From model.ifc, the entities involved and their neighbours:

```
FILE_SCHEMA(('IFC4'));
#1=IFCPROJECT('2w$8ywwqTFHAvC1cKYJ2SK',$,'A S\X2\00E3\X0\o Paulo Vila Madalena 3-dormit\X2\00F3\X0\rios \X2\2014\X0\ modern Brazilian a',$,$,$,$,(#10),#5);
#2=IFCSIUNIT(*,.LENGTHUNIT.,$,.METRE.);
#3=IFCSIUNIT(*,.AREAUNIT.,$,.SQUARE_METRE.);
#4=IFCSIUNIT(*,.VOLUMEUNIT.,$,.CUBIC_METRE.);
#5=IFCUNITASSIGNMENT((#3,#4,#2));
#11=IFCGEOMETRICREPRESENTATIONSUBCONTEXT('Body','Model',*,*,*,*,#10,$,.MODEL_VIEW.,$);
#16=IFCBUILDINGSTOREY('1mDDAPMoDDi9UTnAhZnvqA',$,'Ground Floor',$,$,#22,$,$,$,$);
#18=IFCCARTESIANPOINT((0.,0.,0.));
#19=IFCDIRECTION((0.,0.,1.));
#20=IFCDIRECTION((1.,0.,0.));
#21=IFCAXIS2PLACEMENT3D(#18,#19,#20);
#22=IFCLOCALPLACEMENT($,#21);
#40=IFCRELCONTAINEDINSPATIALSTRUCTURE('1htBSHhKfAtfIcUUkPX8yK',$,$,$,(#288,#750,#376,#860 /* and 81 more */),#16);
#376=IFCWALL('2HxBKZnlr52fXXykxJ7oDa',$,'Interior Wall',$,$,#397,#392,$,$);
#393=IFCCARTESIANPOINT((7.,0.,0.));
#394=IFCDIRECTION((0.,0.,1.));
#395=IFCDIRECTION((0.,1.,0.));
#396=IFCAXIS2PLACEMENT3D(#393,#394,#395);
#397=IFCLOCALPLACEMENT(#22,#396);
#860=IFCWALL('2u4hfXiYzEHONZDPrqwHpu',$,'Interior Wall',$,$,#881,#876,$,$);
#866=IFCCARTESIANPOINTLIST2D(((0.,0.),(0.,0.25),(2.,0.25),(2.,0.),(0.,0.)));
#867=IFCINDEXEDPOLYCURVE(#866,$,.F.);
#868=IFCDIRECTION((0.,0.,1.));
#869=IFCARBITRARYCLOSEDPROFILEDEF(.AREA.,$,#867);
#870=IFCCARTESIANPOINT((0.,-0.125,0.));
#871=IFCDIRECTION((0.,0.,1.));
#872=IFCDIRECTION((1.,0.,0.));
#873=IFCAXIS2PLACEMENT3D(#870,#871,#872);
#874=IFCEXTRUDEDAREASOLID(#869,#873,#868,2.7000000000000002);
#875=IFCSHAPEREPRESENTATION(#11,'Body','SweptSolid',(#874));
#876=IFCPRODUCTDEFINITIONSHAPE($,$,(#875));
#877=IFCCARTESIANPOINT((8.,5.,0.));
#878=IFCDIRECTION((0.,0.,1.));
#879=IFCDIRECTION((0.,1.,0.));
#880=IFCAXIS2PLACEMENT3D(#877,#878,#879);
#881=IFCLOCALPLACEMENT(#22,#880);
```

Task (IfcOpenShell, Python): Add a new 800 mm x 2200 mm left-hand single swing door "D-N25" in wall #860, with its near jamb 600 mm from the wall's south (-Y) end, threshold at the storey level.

```python
import numpy as np
import ifcopenshell
import ifcopenshell.api.feature
import ifcopenshell.api.geometry
import ifcopenshell.api.root
import ifcopenshell.api.spatial
import ifcopenshell.geom
import ifcopenshell.util.element
import ifcopenshell.util.placement
import ifcopenshell.util.representation
import ifcopenshell.util.shape
import ifcopenshell.util.unit

model = ifcopenshell.open("model.ifc")
unit_scale = ifcopenshell.util.unit.calculate_unit_scale(model)
settings = ifcopenshell.geom.settings()


def volume(element):
    """Net volume in cubic metres, openings subtracted."""
    shape = ifcopenshell.geom.create_shape(settings, element)
    return ifcopenshell.util.shape.get_volume(shape.geometry)


wall = model.by_guid("2u4hfXiYzEHONZDPrqwHpu")
storey = ifcopenshell.util.element.get_container(wall, ifc_class="IfcBuildingStorey")
context = ifcopenshell.util.representation.get_context(model, "Model", "Body", "MODEL_VIEW")
before = volume(wall)

width, height, from_end, sill = 0.8, 2.2, 0.6, 0.0  # metres

# The wall runs along its own X axis, and the end named is its -X end.
wall_shape = ifcopenshell.geom.create_shape(settings, wall)
x, y, z = ifcopenshell.util.shape.get_vertices(wall_shape.geometry).T
start = x.min() + from_end
face, thickness = float(y.min()), float(y.max() - y.min())
wall_matrix = ifcopenshell.util.placement.get_local_placement(wall.ObjectPlacement)
level = ifcopenshell.util.placement.get_local_placement(storey.ObjectPlacement)[2, 3]


def in_wall(x, y):
    """Placement at x, y metres in the wall's axes, at sill height."""
    matrix = wall_matrix.copy()
    matrix[:, 3] = wall_matrix @ np.array([x / unit_scale, y / unit_scale, 0.0, 1.0])
    matrix[2, 3] = level + sill / unit_scale
    return matrix


# Opening: a box that overshoots both wall faces by 50 mm.
opening = ifcopenshell.api.root.create_entity(model, ifc_class="IfcOpeningElement", predefined_type="OPENING")
box = ifcopenshell.api.geometry.add_wall_representation(
    model, context=context, length=width, height=height, thickness=thickness + 0.1
)
ifcopenshell.api.geometry.assign_representation(model, product=opening, representation=box)
ifcopenshell.api.geometry.edit_object_placement(model, product=opening, matrix=in_wall(start, face - 0.05), is_si=False)
ifcopenshell.api.feature.add_feature(model, feature=opening, element=wall)

door = ifcopenshell.api.root.create_entity(model, ifc_class="IfcDoor", name="D-N25", predefined_type="DOOR")
door.OverallWidth, door.OverallHeight = width / unit_scale, height / unit_scale
door.OperationType = "SINGLE_SWING_LEFT"
body = ifcopenshell.api.geometry.add_door_representation(
    model,
    context=context,
    overall_width=door.OverallWidth,
    overall_height=door.OverallHeight,
    operation_type="SINGLE_SWING_LEFT",
    lining_properties={"LiningDepth": thickness / unit_scale, "ThresholdDepth": thickness / unit_scale},
)
ifcopenshell.api.geometry.assign_representation(model, product=door, representation=body)
ifcopenshell.api.spatial.assign_container(model, products=[door], relating_structure=storey)
ifcopenshell.api.feature.add_filling(model, opening=opening, element=door)

# The lining spans the wall, so the door starts at the wall face.
ifcopenshell.api.geometry.edit_object_placement(model, product=door, matrix=in_wall(start, face), is_si=False)

after = volume(wall)

print(f"wall volume {before:.3f} -> {after:.3f} m3")

model.write("model_updated.ifc")
```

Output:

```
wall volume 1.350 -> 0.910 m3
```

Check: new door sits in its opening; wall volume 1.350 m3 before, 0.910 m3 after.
